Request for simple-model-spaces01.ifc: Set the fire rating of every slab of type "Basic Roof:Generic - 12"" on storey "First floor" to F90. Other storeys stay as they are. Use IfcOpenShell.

First a look at what the model holds.

```python
import ifcopenshell
import ifcopenshell.util.element

model = ifcopenshell.open("simple-model-spaces01.ifc")
print(model.schema)
storey = next(s for s in model.by_type("IfcBuildingStorey") if s.Name == "First floor")
slabs = [e for e in ifcopenshell.util.element.get_decomposition(storey) if e.is_a("IfcSlab")]
seen = {}
for e in slabs:
    element_type = ifcopenshell.util.element.get_type(e)
    key = (element_type.Name if element_type != e and element_type else None, ifcopenshell.util.element.get_pset(e, "Pset_SlabCommon", "FireRating"))
    seen[key] = seen.get(key, 0) + 1
for (name, value), count in sorted(seen.items(), key=str):
    print(count, "x", name, "|", value)
```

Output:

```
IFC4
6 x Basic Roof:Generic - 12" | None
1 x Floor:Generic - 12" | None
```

```python
import ifcopenshell
import ifcopenshell.api.pset
import ifcopenshell.util.element

model = ifcopenshell.open("simple-model-spaces01.ifc")

storey = next(s for s in model.by_type("IfcBuildingStorey") if s.Name == "First floor")
slabs = [e for e in ifcopenshell.util.element.get_decomposition(storey) if e.is_a("IfcSlab")]

count = 0
for e in slabs:
    element_type = ifcopenshell.util.element.get_type(e)
    if element_type in (None, e) or element_type.Name != 'Basic Roof:Generic - 12"':
        continue
    # add_pset returns the element's existing set when there is one.
    pset = ifcopenshell.api.pset.add_pset(model, product=e, name="Pset_SlabCommon")
    ifcopenshell.api.pset.edit_pset(model, pset=pset, properties={"FireRating": "F90"})
    count += 1

print(count, "slabs updated")

model.write("simple-model-spaces01_updated.ifc")
```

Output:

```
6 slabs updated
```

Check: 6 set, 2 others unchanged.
